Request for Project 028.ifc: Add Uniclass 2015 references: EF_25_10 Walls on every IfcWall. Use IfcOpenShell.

First a look at what the model holds.

```python
import ifcopenshell

model = ifcopenshell.open("Project 028.ifc")
print(model.schema)
print("classifications:", [c.Name for c in model.by_type("IfcClassification")])
for ifc_class in ("IfcDoor", "IfcRoof", "IfcStair", "IfcWall", "IfcWindow"):
    print(ifc_class, len(model.by_type(ifc_class)))
```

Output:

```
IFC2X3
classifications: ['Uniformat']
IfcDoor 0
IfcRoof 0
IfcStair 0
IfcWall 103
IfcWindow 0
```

```python
import ifcopenshell
import ifcopenshell.api.classification

model = ifcopenshell.open("Project 028.ifc")

# IFC2X3 requires Source and Edition and has no link from the project to the system.
system = model.create_entity("IfcClassification", Source="NBS", Edition="2015", Name="Uniclass 2015")

codes = {
    "IfcWall": ("EF_25_10", "Walls"),
}
for ifc_class, (code, name) in codes.items():
    products = model.by_type(ifc_class)
    ifcopenshell.api.classification.add_reference(
        model, products=products, classification=system, identification=code, name=name
    )
    print(code, len(products))

model.write("Project 028_v2.ifc")
```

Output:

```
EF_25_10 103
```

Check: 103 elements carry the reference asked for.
